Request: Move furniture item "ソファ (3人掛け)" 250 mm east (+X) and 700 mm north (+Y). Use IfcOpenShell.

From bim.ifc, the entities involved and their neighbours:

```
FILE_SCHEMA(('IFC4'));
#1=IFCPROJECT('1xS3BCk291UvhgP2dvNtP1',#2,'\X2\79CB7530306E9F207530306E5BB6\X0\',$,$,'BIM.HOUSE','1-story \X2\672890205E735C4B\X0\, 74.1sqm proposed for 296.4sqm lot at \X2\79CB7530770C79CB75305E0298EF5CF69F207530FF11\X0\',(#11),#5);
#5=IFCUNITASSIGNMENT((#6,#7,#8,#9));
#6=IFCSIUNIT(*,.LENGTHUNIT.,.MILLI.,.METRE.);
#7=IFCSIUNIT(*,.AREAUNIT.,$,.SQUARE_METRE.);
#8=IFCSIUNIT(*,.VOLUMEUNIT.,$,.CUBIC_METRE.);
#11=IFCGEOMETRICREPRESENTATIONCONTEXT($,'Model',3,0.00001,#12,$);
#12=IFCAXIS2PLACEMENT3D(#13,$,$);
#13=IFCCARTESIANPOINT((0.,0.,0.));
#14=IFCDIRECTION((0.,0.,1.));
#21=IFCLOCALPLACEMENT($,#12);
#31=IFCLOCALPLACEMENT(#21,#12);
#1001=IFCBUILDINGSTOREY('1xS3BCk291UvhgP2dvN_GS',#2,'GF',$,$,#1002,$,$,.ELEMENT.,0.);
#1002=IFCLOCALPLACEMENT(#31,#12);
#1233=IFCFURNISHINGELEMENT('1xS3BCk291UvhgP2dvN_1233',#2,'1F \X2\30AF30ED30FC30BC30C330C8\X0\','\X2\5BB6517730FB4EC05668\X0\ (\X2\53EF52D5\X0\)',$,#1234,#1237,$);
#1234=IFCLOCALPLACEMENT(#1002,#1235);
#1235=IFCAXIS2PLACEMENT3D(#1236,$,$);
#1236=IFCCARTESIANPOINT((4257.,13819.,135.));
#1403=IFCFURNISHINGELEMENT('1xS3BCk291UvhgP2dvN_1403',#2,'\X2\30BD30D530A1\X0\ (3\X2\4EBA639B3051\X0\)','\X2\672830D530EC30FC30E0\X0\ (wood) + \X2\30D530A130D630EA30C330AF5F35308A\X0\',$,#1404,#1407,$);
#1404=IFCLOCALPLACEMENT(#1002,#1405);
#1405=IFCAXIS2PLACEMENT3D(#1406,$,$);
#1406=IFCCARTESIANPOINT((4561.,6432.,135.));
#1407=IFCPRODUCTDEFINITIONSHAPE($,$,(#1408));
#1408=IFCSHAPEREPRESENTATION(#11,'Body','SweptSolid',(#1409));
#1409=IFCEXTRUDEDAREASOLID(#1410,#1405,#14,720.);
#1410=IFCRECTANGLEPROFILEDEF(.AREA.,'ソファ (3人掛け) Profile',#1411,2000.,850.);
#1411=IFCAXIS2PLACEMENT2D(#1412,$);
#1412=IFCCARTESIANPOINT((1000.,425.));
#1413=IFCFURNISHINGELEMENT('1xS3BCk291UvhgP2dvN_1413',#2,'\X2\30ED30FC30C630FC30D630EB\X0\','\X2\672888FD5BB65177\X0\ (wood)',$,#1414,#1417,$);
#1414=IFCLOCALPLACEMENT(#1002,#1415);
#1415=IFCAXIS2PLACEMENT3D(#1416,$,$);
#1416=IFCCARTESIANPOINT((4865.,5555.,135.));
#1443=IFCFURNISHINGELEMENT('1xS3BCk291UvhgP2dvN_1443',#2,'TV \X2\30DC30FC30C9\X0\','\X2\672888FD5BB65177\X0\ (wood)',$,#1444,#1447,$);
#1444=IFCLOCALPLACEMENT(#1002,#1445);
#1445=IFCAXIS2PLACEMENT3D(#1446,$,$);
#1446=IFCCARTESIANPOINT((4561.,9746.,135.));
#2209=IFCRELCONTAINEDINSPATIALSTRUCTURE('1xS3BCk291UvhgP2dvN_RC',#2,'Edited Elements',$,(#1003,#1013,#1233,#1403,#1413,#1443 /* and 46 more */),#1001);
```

```python
import ifcopenshell
import ifcopenshell.api.geometry
import ifcopenshell.util.placement
import ifcopenshell.util.unit

model = ifcopenshell.open("bim.ifc")
unit_scale = ifcopenshell.util.unit.calculate_unit_scale(model)

item = model.by_guid("1xS3BCk291UvhgP2dvN_1403")
matrix = ifcopenshell.util.placement.get_local_placement(item.ObjectPlacement)
matrix[0, 3] += 0.25 / unit_scale
matrix[1, 3] += 0.7 / unit_scale
ifcopenshell.api.geometry.edit_object_placement(model, product=item, matrix=matrix, is_si=False)

print(ifcopenshell.util.placement.get_local_placement(item.ObjectPlacement).round(3) + 0.0)

model.write("bim-out.ifc")
```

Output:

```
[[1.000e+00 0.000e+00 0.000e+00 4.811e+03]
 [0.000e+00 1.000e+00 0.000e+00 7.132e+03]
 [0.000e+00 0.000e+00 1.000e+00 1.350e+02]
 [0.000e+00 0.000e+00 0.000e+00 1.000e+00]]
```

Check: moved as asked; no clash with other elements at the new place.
